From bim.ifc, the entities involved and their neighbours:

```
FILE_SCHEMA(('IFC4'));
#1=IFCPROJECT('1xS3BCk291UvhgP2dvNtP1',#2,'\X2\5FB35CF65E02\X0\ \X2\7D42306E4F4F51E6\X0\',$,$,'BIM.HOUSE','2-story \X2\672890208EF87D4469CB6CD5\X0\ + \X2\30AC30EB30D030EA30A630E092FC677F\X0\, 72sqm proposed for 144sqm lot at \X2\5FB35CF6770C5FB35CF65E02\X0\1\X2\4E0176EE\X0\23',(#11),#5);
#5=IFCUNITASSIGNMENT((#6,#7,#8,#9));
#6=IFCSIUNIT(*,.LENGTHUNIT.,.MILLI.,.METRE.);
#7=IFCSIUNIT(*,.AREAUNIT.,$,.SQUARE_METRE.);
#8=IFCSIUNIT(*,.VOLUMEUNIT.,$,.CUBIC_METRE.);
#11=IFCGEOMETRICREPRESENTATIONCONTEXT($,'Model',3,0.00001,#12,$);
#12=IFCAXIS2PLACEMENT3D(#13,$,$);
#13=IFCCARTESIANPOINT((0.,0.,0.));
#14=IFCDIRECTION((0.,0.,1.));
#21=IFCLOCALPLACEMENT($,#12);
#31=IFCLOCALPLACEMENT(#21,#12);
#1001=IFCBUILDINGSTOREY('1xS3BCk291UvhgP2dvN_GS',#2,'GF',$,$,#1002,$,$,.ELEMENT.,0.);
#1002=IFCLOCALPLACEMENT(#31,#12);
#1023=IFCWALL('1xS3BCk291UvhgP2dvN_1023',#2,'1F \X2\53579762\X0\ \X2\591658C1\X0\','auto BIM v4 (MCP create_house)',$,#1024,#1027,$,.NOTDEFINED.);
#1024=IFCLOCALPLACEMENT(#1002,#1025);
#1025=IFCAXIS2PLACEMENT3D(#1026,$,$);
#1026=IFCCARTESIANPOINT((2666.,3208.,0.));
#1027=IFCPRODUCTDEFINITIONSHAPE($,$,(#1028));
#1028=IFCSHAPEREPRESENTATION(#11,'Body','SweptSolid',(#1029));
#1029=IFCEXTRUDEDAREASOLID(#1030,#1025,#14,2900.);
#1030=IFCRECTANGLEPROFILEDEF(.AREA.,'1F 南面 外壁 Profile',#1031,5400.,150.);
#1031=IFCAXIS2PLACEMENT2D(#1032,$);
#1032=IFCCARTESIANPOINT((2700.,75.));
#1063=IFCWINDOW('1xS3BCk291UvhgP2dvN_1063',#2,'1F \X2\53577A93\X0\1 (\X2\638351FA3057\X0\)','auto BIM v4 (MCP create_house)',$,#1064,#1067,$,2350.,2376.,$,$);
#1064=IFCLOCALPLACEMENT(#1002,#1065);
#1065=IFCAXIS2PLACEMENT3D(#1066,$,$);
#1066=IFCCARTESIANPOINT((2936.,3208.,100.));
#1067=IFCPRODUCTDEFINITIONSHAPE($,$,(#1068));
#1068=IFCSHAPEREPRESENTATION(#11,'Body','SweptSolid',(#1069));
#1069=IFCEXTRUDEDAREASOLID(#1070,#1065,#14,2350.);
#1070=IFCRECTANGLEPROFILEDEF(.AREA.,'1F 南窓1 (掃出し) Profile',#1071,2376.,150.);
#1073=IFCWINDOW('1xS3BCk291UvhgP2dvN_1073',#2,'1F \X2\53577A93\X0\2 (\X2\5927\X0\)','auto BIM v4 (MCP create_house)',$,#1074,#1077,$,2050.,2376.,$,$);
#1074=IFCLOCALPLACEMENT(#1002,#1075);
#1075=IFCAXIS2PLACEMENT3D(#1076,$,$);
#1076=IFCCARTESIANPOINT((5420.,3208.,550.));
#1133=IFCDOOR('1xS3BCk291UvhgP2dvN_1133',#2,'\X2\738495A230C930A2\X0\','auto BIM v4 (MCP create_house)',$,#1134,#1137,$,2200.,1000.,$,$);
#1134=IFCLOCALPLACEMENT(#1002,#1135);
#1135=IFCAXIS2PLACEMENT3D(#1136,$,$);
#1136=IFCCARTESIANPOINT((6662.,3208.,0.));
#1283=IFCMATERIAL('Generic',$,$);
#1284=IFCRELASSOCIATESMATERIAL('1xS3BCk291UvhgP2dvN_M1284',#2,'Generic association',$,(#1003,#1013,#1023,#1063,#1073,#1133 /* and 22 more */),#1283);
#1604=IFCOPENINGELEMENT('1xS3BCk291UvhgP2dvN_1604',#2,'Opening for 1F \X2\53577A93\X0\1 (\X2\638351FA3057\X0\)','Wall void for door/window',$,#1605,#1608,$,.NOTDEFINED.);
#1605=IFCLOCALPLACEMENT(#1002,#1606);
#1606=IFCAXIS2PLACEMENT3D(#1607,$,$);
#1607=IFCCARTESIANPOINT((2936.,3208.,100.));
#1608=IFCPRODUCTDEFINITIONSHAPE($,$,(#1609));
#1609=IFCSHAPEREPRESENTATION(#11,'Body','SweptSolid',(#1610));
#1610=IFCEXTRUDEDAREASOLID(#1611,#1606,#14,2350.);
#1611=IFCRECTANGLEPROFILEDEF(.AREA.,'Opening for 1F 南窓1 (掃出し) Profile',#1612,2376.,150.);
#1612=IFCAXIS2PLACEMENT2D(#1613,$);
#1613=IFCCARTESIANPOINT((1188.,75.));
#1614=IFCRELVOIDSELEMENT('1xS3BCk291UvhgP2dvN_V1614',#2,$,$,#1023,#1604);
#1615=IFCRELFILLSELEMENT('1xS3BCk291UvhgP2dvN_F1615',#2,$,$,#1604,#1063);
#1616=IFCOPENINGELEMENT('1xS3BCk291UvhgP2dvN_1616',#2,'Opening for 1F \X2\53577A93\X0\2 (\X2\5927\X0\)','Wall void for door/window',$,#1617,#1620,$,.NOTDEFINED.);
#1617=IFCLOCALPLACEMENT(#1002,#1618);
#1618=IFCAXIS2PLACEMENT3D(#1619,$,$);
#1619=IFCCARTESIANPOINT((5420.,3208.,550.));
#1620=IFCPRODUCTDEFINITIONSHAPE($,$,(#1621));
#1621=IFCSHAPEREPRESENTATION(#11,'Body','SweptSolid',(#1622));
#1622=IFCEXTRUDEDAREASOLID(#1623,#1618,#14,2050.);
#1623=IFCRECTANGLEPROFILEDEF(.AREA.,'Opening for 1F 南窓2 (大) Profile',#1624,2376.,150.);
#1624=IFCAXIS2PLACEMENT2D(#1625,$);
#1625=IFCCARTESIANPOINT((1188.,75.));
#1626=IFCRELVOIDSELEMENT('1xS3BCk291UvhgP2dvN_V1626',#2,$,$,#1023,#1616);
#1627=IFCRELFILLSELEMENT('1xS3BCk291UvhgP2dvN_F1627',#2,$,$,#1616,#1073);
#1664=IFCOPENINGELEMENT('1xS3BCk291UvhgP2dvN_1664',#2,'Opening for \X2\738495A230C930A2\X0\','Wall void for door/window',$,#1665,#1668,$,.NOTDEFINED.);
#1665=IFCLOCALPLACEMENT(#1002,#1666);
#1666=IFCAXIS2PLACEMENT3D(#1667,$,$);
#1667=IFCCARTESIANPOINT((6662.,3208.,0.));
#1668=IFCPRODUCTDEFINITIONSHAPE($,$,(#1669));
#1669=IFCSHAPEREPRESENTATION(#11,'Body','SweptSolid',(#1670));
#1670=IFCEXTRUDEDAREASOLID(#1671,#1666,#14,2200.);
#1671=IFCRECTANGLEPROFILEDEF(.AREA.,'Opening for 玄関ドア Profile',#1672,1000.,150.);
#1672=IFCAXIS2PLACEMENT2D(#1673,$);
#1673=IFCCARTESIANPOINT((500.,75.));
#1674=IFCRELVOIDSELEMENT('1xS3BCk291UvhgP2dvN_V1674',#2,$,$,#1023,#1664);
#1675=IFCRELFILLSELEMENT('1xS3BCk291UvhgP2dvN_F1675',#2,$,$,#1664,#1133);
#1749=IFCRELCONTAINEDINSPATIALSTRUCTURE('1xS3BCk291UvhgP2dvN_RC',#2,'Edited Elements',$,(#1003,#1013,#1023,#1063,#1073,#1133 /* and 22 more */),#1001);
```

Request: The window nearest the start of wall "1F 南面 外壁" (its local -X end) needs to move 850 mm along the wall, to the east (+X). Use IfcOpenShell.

```python
import ifcopenshell
import ifcopenshell.api.geometry
import ifcopenshell.util.placement

model = ifcopenshell.open("bim.ifc")

window = model.by_id(1063)
opening = window.FillsVoids[0].RelatingOpeningElement
wall = opening.VoidsElements[0].RelatingBuildingElement

wall_matrix = ifcopenshell.util.placement.get_local_placement(wall.ObjectPlacement)
shift = wall_matrix[:3, 0] * 850.0
before = ifcopenshell.util.placement.get_local_placement(window.ObjectPlacement)[:3, 3].copy()

# The window is not placed relative to its opening, so move both.
for product in (opening, window):
    matrix = ifcopenshell.util.placement.get_local_placement(product.ObjectPlacement)
    matrix[:3, 3] += shift
    ifcopenshell.api.geometry.edit_object_placement(model, product=product, matrix=matrix, is_si=False)

after = ifcopenshell.util.placement.get_local_placement(window.ObjectPlacement)[:3, 3]
print("window moved by", (after - before).round(3) + 0.0)

model.write("bim-out.ifc")
```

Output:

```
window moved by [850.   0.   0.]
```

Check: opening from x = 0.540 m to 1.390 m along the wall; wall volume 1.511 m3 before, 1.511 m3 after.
